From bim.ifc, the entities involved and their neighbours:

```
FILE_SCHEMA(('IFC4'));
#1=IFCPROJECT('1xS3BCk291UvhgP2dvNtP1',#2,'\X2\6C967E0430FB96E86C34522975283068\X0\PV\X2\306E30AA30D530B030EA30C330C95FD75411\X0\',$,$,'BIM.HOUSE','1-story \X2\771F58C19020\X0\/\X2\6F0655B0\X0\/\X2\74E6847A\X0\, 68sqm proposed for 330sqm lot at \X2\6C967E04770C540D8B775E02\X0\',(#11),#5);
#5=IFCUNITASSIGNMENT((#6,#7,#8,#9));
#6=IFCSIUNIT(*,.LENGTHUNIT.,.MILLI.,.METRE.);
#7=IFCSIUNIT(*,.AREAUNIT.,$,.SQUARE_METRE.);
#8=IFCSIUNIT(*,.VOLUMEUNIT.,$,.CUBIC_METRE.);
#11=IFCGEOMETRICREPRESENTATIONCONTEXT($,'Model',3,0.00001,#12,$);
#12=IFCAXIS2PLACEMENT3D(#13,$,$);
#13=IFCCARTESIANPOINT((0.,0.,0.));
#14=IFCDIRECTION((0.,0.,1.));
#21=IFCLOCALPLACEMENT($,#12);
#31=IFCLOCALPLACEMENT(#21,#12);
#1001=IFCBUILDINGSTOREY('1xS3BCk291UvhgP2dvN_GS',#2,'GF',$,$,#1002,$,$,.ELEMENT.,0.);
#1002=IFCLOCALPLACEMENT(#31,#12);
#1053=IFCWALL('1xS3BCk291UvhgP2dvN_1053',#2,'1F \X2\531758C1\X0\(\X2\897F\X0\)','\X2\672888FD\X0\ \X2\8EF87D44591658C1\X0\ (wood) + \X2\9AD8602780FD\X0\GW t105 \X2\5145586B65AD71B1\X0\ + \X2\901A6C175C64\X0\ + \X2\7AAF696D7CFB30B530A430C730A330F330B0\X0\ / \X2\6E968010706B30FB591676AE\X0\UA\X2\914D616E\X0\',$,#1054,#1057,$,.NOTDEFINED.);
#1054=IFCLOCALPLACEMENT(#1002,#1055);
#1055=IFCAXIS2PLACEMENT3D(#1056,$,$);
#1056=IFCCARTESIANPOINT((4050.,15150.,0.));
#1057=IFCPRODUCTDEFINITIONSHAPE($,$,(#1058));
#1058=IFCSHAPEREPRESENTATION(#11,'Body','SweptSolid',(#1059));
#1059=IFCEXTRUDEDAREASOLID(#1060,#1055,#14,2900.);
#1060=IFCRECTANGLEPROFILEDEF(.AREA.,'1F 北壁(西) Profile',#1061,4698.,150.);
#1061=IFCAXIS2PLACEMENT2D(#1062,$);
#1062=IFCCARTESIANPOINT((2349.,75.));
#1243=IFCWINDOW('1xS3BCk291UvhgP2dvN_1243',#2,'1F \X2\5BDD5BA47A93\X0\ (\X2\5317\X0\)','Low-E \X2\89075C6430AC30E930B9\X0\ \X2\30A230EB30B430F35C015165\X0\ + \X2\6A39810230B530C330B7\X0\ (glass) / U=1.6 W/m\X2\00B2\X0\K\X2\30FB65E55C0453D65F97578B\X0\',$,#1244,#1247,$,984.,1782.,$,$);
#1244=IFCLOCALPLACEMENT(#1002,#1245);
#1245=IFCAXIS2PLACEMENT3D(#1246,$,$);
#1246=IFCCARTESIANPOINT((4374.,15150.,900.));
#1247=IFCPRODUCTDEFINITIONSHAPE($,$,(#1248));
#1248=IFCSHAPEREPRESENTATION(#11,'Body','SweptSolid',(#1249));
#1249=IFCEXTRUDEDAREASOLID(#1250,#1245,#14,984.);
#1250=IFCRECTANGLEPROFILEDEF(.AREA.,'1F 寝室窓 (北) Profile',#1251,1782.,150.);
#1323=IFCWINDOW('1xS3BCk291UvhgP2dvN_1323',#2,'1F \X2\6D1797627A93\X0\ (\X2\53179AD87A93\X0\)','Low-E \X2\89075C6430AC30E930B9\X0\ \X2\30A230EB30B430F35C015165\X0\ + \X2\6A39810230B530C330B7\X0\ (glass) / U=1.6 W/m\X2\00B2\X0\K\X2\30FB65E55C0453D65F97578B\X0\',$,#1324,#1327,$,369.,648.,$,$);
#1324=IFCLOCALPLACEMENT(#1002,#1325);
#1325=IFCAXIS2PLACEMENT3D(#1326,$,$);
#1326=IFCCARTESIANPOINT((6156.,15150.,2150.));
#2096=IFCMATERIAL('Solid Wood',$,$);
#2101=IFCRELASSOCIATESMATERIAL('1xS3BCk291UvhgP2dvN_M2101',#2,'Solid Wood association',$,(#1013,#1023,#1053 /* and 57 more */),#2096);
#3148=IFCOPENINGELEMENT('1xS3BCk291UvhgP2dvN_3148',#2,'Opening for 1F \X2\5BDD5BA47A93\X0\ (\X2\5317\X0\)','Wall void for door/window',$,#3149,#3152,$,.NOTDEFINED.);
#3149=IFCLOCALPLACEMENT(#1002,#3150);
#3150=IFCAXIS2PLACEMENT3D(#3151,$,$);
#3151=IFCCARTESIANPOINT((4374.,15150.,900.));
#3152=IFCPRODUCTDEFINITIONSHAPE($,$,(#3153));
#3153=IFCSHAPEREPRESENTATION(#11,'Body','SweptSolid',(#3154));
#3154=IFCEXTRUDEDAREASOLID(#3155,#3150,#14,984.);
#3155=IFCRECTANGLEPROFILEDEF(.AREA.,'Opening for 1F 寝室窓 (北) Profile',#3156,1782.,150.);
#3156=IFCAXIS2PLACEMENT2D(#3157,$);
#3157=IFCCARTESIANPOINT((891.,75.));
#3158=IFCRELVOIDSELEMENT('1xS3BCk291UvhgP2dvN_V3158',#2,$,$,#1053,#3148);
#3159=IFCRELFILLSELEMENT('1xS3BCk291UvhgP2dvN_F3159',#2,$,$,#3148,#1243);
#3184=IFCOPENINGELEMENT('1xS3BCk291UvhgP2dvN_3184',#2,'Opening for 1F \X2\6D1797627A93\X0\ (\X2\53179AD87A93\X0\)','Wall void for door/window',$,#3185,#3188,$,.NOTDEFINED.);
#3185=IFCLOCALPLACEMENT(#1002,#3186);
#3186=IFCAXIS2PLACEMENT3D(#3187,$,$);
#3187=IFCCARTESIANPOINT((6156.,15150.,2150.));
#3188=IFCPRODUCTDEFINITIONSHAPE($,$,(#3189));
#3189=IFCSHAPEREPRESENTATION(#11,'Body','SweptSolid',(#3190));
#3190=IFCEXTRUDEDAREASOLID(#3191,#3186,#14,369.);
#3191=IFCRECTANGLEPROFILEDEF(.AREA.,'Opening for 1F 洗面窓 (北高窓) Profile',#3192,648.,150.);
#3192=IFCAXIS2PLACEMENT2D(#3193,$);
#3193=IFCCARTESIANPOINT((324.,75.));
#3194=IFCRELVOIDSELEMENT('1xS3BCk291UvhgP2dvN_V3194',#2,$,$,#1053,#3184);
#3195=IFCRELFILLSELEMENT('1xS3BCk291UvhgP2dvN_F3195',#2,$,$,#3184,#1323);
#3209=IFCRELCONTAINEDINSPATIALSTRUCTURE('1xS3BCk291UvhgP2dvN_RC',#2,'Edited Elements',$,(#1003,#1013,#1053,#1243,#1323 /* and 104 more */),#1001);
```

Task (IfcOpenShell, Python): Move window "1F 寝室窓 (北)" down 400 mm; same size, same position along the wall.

```python
import numpy as np
import ifcopenshell
import ifcopenshell.api.geometry
import ifcopenshell.util.placement
import ifcopenshell.util.unit

model = ifcopenshell.open("bim.ifc")
unit_scale = ifcopenshell.util.unit.calculate_unit_scale(model)

window = model.by_id(1243)
opening = window.FillsVoids[0].RelatingOpeningElement
dz = -0.4 / unit_scale

shift = np.array([0.0, 0.0, dz])
# The window is not placed relative to its opening, so move both.
for product in (opening, window):
    matrix = ifcopenshell.util.placement.get_local_placement(product.ObjectPlacement)
    matrix[:3, 3] += shift
    ifcopenshell.api.geometry.edit_object_placement(model, product=product, matrix=matrix, is_si=False)

print(f"moved by {dz * unit_scale:+.3f} m")

model.write("bim_v2.ifc")
```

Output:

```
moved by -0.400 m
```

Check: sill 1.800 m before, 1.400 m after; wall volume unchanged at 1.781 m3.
